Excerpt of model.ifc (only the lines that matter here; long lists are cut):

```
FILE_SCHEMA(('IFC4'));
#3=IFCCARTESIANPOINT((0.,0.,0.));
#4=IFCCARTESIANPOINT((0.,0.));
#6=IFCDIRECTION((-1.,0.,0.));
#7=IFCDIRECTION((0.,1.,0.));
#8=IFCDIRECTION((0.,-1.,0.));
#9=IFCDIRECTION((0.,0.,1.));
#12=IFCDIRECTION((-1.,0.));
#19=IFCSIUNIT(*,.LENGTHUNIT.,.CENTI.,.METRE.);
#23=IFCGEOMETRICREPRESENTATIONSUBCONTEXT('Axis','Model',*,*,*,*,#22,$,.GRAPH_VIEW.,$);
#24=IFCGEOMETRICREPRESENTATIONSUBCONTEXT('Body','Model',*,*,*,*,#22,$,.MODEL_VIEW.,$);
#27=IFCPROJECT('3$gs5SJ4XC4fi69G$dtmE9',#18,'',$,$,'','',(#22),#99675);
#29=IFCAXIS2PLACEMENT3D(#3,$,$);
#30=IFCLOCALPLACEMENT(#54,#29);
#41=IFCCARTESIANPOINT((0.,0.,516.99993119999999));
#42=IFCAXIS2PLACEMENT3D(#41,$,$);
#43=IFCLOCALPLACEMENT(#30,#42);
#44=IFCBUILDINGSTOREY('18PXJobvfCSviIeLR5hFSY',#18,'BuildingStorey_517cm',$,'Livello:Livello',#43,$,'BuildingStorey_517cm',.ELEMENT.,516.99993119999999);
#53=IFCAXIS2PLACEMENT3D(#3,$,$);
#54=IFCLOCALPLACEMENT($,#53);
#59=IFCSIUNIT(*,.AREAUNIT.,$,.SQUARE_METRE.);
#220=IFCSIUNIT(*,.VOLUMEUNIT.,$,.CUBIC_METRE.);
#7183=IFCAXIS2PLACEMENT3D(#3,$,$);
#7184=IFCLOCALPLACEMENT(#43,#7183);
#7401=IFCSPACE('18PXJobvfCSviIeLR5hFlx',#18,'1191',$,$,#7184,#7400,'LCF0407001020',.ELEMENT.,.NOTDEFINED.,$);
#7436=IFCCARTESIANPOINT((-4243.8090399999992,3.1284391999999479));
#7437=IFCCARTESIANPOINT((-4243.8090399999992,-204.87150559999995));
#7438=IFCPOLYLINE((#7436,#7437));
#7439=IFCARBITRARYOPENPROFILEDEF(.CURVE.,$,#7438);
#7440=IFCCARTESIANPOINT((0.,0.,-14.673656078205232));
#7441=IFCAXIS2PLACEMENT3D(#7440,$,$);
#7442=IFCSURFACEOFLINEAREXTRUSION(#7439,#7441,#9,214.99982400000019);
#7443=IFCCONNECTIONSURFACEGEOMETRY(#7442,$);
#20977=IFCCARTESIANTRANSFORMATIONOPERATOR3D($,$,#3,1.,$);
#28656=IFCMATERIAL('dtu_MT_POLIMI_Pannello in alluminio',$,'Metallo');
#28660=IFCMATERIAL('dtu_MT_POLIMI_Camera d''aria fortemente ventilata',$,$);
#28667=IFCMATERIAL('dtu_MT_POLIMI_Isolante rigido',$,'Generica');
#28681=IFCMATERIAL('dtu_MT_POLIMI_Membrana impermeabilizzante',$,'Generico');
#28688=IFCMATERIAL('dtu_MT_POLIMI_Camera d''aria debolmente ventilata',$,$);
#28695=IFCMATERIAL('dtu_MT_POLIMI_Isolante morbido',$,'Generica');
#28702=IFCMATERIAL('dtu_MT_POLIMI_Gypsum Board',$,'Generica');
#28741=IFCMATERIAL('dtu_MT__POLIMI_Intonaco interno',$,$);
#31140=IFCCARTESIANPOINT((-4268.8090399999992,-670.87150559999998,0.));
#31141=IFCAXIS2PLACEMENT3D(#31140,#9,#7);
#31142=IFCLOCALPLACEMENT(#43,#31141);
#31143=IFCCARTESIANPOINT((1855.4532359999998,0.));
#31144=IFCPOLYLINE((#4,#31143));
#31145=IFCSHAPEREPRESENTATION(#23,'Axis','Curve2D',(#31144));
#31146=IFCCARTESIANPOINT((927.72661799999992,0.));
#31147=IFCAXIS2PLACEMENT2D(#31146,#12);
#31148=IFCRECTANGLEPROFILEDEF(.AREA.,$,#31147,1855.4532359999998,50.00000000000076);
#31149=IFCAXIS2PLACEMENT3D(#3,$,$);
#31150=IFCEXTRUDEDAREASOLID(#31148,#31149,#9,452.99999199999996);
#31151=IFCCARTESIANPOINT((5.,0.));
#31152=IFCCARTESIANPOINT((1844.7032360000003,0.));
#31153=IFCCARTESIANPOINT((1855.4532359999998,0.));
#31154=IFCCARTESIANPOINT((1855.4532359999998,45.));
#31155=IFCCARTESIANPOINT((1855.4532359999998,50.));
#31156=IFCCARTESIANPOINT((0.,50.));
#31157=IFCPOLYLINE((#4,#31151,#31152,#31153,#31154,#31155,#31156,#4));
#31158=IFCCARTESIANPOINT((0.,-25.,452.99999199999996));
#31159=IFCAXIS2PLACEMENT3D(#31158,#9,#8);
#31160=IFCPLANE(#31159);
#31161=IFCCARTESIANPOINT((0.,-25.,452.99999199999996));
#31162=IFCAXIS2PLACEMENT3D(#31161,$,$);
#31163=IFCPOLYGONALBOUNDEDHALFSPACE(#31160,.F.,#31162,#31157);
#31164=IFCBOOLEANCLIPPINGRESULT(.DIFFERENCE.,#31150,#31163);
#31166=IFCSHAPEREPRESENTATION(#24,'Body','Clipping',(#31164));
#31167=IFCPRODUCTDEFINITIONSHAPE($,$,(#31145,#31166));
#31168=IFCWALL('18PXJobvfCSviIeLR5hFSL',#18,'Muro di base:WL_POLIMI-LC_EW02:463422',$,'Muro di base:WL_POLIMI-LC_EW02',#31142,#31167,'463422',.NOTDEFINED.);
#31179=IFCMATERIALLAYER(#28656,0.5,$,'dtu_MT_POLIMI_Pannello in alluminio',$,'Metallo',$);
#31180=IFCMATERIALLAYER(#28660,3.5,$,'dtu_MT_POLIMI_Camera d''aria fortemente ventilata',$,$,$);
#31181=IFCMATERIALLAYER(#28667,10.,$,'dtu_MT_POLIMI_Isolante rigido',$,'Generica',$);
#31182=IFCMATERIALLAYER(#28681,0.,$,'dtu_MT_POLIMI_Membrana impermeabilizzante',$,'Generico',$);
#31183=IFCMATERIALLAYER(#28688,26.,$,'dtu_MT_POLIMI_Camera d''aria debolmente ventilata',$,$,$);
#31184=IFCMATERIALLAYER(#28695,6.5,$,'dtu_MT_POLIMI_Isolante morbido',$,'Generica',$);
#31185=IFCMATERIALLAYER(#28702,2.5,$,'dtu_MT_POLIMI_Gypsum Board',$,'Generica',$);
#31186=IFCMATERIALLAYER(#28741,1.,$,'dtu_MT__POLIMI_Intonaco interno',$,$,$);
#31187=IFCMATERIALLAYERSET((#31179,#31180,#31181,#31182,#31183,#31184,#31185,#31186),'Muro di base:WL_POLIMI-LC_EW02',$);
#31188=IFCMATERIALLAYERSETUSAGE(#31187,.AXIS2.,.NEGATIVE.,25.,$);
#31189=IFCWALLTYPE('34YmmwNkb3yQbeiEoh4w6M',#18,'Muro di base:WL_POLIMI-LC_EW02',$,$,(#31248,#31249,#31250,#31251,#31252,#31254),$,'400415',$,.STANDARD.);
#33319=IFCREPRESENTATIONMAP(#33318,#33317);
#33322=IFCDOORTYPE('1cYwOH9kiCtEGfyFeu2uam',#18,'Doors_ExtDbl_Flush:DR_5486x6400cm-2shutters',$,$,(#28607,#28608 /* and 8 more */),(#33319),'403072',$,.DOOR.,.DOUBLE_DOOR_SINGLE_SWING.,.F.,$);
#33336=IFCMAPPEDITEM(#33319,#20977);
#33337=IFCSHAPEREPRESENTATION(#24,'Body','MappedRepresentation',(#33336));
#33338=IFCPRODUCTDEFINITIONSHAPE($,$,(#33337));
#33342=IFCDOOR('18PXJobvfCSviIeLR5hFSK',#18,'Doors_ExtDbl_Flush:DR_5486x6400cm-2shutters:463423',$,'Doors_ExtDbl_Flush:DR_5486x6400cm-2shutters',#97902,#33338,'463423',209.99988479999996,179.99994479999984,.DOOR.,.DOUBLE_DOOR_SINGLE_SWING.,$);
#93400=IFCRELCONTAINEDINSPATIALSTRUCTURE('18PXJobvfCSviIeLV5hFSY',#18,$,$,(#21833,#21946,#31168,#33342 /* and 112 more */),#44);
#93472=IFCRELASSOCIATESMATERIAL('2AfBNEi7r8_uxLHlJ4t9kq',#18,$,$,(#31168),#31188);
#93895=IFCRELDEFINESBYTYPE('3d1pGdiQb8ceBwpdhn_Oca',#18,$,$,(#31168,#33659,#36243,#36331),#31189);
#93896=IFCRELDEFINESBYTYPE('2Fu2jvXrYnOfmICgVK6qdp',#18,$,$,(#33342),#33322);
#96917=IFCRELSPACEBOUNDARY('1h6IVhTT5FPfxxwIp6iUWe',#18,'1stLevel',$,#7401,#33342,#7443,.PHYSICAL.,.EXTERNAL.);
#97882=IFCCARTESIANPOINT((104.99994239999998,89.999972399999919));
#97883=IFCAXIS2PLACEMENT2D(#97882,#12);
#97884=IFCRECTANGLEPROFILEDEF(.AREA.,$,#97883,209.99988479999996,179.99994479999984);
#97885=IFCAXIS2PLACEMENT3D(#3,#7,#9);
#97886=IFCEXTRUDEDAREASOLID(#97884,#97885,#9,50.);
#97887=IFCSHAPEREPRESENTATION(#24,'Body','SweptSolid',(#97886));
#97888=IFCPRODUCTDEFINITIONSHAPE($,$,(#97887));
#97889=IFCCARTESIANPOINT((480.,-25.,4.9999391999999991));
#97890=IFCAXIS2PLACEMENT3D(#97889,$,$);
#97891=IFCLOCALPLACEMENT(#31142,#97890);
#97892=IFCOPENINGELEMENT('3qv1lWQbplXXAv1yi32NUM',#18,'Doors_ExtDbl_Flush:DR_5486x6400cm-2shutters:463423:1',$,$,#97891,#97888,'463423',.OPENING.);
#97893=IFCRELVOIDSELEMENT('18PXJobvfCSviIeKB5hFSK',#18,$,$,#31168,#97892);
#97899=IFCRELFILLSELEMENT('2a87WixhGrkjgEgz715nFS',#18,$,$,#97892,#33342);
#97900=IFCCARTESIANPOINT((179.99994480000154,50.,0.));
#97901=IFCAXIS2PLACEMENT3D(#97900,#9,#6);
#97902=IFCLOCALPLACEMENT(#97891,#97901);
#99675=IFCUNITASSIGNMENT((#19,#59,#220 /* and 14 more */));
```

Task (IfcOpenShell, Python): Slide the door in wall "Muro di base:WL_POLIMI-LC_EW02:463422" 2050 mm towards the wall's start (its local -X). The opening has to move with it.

```python
import numpy as np
import ifcopenshell
import ifcopenshell.api.geometry
import ifcopenshell.util.placement
import ifcopenshell.util.unit

model = ifcopenshell.open("model.ifc")
unit_scale = ifcopenshell.util.unit.calculate_unit_scale(model)

door = model.by_guid("18PXJobvfCSviIeLR5hFSK")
opening = door.FillsVoids[0].RelatingOpeningElement
wall = opening.VoidsElements[0].RelatingBuildingElement

wall_matrix = ifcopenshell.util.placement.get_local_placement(wall.ObjectPlacement)
shift = wall_matrix[:3, 0] * -2.05 / unit_scale
before = ifcopenshell.util.placement.get_local_placement(door.ObjectPlacement)[:3, 3].copy()

# The door is placed relative to its opening, so it follows when the opening moves.
matrix = ifcopenshell.util.placement.get_local_placement(opening.ObjectPlacement)
matrix[:3, 3] += shift
ifcopenshell.api.geometry.edit_object_placement(
    model, product=opening, matrix=matrix, is_si=False, should_transform_children=True
)

# Space boundary surfaces are stored in each space's coordinates; move them too.
for rel in door.ProvidesBoundaries:
    if not rel.ConnectionGeometry:
        continue
    surface = rel.ConnectionGeometry.SurfaceOnRelatingElement
    space_matrix = ifcopenshell.util.placement.get_local_placement(rel.RelatingSpace.ObjectPlacement)
    point = np.array(surface.Position.Location.Coordinates) + space_matrix[:3, :3].T @ shift
    surface.Position = model.createIfcAxis2Placement3D(
        model.createIfcCartesianPoint(point.tolist()), surface.Position.Axis, surface.Position.RefDirection
    )

after = ifcopenshell.util.placement.get_local_placement(door.ObjectPlacement)[:3, 3]
print("door moved by", (after - before).round(3) + 0.0)

model.write("model_v2.ifc")
```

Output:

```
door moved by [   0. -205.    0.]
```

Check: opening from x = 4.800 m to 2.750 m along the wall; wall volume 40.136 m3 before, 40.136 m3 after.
